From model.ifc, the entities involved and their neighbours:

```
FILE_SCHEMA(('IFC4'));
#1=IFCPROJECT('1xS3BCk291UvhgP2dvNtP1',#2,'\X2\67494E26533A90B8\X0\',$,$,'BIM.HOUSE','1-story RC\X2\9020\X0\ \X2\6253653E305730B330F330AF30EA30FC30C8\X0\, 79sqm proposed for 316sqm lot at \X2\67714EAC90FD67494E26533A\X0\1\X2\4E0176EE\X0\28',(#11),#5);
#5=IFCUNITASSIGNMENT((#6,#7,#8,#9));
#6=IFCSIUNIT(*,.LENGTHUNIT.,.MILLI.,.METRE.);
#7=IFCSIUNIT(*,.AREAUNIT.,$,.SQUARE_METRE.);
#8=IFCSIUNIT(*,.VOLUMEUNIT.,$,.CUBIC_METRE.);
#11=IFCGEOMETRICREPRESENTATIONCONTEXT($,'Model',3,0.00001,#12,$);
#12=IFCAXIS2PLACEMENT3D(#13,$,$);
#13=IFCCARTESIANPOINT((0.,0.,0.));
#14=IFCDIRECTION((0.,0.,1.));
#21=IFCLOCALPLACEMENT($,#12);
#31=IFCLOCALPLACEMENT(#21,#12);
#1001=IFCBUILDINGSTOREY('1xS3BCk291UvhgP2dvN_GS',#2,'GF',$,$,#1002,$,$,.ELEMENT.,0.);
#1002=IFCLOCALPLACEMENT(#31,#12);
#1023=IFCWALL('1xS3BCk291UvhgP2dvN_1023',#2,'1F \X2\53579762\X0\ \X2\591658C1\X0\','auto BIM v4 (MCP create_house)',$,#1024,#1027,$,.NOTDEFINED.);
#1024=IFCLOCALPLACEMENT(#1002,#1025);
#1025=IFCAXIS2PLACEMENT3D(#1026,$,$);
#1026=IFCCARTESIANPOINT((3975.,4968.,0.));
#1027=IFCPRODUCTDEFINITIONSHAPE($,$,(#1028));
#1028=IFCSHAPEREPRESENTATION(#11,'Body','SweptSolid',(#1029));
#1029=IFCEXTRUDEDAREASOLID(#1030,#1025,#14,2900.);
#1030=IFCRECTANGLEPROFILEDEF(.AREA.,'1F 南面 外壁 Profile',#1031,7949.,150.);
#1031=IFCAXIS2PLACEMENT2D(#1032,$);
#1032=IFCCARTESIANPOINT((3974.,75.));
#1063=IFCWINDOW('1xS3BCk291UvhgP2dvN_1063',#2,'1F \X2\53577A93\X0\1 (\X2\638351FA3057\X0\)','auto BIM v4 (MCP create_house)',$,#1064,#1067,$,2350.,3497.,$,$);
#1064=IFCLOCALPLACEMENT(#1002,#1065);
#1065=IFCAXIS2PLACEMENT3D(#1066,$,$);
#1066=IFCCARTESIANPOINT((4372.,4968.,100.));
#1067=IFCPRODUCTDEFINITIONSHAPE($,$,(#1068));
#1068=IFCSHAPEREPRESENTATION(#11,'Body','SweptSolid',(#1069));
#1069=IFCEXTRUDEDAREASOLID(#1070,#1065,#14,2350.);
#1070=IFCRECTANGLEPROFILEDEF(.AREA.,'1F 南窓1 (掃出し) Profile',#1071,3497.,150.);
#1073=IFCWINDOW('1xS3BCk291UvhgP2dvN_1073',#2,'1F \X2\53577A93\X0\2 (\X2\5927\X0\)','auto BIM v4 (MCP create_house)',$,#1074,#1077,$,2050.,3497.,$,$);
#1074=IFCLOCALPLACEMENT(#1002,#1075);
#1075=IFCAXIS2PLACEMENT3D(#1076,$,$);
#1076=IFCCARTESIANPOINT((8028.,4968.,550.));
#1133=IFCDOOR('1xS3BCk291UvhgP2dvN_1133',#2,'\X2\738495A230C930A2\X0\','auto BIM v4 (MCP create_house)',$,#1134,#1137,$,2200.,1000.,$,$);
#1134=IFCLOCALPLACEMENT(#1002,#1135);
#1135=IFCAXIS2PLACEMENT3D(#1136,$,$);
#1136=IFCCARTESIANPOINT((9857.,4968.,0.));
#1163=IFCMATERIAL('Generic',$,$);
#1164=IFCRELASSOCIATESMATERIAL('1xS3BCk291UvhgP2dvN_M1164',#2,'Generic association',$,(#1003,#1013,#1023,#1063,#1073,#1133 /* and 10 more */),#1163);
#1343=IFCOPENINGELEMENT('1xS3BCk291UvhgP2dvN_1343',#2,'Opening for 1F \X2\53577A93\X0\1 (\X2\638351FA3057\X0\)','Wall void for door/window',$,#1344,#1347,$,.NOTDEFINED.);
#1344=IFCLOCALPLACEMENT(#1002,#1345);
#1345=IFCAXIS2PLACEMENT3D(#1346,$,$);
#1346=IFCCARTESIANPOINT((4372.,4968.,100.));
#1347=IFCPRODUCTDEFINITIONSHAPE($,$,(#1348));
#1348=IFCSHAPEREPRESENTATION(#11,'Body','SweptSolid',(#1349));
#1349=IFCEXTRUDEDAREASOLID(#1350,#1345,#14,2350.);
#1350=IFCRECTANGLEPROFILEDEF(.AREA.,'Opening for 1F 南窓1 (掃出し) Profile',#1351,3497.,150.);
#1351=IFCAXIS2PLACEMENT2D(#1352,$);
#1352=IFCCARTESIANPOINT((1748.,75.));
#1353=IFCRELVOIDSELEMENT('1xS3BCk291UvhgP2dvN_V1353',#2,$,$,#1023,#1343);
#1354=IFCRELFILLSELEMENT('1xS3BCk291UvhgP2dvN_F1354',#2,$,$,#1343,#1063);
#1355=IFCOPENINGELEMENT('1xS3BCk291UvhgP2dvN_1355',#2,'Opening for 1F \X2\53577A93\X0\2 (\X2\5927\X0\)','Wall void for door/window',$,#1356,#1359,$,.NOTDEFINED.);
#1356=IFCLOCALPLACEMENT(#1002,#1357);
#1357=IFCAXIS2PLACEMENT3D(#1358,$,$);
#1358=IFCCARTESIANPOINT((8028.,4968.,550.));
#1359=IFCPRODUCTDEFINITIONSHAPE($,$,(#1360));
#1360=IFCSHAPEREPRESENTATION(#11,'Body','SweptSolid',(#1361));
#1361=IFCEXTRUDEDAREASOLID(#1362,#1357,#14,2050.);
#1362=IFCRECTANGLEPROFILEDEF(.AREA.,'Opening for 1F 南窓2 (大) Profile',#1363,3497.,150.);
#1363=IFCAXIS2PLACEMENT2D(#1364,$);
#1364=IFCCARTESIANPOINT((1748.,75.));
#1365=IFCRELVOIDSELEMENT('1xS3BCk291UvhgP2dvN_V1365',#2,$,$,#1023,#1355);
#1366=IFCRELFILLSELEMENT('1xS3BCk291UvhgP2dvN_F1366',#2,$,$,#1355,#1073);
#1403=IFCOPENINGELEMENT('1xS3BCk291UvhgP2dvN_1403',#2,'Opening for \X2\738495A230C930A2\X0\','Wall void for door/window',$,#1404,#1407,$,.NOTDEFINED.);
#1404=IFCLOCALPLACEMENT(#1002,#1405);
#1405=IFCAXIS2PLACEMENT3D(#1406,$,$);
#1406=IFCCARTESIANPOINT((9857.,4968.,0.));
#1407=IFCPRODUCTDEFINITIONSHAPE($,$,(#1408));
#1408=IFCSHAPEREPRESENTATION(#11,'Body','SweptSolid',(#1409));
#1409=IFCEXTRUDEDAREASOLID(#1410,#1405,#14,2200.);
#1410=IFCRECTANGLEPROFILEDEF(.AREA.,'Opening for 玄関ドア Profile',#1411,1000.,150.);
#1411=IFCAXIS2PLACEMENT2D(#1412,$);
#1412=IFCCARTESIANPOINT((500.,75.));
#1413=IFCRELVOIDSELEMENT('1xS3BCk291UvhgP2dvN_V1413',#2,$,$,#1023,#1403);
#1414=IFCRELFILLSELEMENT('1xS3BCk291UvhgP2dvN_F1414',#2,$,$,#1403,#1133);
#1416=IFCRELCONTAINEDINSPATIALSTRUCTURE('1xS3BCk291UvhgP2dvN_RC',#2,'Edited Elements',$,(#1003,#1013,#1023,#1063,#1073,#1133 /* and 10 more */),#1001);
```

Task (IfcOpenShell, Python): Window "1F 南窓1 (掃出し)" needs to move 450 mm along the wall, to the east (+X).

```python
import ifcopenshell
import ifcopenshell.api.geometry
import ifcopenshell.util.placement
import ifcopenshell.util.unit

model = ifcopenshell.open("model.ifc")
unit_scale = ifcopenshell.util.unit.calculate_unit_scale(model)

window = model.by_id(1063)
opening = window.FillsVoids[0].RelatingOpeningElement
wall = opening.VoidsElements[0].RelatingBuildingElement

wall_matrix = ifcopenshell.util.placement.get_local_placement(wall.ObjectPlacement)
shift = wall_matrix[:3, 0] * 0.45 / unit_scale
before = ifcopenshell.util.placement.get_local_placement(window.ObjectPlacement)[:3, 3].copy()

# The window is not placed relative to its opening, so move both.
for product in (opening, window):
    matrix = ifcopenshell.util.placement.get_local_placement(product.ObjectPlacement)
    matrix[:3, 3] += shift
    ifcopenshell.api.geometry.edit_object_placement(model, product=product, matrix=matrix, is_si=False)

after = ifcopenshell.util.placement.get_local_placement(window.ObjectPlacement)[:3, 3]
print("window moved by", (after - before).round(3) + 0.0)

model.write("model_v2.ifc")
```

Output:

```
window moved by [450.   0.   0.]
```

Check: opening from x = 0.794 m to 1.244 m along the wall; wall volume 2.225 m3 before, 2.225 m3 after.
